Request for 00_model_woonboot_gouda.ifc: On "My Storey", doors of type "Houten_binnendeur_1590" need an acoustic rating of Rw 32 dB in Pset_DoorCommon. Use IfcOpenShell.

First a look at what the model holds.

```python
import ifcopenshell
import ifcopenshell.util.element

model = ifcopenshell.open("00_model_woonboot_gouda.ifc")
print(model.schema)
storey = next(s for s in model.by_type("IfcBuildingStorey") if s.Name == "My Storey")
doors = [e for e in ifcopenshell.util.element.get_decomposition(storey) if e.is_a("IfcDoor")]
seen = {}
for e in doors:
    element_type = ifcopenshell.util.element.get_type(e)
    key = (element_type.Name if element_type != e and element_type else None, ifcopenshell.util.element.get_pset(e, "Pset_DoorCommon", "AcousticRating"))
    seen[key] = seen.get(key, 0) + 1
for (name, value), count in sorted(seen.items(), key=str):
    print(count, "x", name, "|", value)
```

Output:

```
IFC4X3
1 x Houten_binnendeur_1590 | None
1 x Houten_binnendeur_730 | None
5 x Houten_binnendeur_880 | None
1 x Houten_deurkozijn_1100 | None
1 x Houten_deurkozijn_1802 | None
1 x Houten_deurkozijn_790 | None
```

```python
import ifcopenshell
import ifcopenshell.api.pset
import ifcopenshell.util.element

model = ifcopenshell.open("00_model_woonboot_gouda.ifc")

storey = next(s for s in model.by_type("IfcBuildingStorey") if s.Name == "My Storey")
doors = [e for e in ifcopenshell.util.element.get_decomposition(storey) if e.is_a("IfcDoor")]

count = 0
for e in doors:
    element_type = ifcopenshell.util.element.get_type(e)
    if element_type in (None, e) or element_type.Name != "Houten_binnendeur_1590":
        continue
    # add_pset returns the element's existing set when there is one.
    pset = ifcopenshell.api.pset.add_pset(model, product=e, name="Pset_DoorCommon")
    ifcopenshell.api.pset.edit_pset(model, pset=pset, properties={"AcousticRating": "Rw 32 dB"})
    count += 1

print(count, "doors updated")

model.write("00_model_woonboot_gouda_rev.ifc")
```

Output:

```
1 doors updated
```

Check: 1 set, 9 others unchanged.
